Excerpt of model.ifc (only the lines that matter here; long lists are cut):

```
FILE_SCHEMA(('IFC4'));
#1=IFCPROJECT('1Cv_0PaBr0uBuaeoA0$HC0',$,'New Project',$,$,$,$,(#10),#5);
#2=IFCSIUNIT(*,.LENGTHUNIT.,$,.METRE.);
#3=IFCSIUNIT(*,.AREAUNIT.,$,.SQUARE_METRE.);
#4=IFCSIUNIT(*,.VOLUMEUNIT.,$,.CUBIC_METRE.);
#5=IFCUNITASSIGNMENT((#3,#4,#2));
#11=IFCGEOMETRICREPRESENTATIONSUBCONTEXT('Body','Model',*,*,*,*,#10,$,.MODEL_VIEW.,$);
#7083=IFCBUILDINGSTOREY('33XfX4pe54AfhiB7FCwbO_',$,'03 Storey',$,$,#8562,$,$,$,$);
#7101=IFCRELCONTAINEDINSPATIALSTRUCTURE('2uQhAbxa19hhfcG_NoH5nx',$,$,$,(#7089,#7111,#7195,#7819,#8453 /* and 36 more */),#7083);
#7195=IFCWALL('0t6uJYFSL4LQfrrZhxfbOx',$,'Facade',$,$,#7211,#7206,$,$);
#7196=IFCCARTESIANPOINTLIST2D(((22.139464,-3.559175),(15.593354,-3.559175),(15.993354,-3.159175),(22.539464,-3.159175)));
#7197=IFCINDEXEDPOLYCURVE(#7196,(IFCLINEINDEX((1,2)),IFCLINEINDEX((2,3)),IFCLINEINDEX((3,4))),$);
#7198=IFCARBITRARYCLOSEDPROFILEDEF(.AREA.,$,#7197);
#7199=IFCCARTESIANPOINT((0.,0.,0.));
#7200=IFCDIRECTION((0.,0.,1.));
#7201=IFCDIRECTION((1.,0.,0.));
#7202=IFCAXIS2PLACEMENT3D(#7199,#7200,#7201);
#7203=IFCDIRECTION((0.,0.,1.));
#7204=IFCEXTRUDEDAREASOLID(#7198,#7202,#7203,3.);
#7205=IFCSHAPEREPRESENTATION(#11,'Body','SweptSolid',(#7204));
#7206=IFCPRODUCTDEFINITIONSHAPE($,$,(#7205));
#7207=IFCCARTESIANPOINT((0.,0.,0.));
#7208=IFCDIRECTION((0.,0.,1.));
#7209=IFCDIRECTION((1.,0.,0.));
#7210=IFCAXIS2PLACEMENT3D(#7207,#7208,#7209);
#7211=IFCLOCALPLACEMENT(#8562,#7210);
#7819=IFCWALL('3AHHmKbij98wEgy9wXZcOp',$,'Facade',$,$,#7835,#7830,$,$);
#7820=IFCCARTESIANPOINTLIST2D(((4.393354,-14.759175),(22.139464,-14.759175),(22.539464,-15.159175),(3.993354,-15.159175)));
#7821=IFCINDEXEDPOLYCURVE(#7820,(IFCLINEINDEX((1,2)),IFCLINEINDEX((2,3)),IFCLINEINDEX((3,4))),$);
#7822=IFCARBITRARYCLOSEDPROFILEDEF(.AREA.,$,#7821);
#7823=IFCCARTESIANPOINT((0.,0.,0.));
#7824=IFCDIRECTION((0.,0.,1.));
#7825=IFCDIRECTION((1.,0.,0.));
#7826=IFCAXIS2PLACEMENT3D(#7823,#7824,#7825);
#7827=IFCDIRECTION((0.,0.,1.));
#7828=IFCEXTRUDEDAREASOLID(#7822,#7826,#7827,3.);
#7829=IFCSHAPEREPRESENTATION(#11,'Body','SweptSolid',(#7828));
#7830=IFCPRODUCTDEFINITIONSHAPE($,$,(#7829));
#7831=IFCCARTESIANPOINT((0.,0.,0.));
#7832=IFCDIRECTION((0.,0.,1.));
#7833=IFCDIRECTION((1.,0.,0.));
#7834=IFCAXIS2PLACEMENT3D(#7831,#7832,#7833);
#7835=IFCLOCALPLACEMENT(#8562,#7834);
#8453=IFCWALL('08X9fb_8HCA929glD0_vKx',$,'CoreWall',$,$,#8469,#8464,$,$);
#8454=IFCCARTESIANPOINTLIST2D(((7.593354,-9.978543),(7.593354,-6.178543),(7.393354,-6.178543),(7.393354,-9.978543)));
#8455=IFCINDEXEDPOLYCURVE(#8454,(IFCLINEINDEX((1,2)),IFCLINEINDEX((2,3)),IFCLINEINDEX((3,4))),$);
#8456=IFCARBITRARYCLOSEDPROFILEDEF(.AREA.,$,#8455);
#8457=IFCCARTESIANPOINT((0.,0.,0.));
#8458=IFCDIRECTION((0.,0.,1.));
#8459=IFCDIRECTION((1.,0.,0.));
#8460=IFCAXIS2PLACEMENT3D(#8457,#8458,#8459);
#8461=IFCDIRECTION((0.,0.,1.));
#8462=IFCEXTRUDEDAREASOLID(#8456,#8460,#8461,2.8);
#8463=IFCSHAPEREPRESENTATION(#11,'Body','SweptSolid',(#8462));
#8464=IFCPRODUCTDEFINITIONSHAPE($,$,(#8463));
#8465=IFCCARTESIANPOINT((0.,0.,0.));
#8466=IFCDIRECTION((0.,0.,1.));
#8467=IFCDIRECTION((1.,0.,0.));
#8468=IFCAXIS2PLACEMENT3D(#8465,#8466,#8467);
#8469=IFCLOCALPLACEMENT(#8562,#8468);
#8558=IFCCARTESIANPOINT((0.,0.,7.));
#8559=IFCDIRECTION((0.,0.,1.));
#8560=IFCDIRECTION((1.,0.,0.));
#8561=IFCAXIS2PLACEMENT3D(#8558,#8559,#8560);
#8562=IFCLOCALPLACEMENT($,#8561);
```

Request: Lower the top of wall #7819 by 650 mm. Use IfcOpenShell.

```python
import ifcopenshell
import ifcopenshell.geom
import ifcopenshell.util.representation
import ifcopenshell.util.shape
import ifcopenshell.util.unit

model = ifcopenshell.open("model.ifc")
unit_scale = ifcopenshell.util.unit.calculate_unit_scale(model)
settings = ifcopenshell.geom.settings()


def volume(element):
    """Net volume in cubic metres, openings subtracted."""
    shape = ifcopenshell.geom.create_shape(settings, element)
    return ifcopenshell.util.shape.get_volume(shape.geometry)


wall = model.by_guid("3AHHmKbij98wEgy9wXZcOp")
before = volume(wall)

body = ifcopenshell.util.representation.get_representation(wall, "Model", "Body")
solid = body.Items[0]
old_height = solid.Depth
solid.Depth -= 0.65 / unit_scale
after = volume(wall)

print(f"height {old_height:g} -> {solid.Depth:g}, volume {before:.3f} -> {after:.3f} m3")

model.write("model-out.ifc")
```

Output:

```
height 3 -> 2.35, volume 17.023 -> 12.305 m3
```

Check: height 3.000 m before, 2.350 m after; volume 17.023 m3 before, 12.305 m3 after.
